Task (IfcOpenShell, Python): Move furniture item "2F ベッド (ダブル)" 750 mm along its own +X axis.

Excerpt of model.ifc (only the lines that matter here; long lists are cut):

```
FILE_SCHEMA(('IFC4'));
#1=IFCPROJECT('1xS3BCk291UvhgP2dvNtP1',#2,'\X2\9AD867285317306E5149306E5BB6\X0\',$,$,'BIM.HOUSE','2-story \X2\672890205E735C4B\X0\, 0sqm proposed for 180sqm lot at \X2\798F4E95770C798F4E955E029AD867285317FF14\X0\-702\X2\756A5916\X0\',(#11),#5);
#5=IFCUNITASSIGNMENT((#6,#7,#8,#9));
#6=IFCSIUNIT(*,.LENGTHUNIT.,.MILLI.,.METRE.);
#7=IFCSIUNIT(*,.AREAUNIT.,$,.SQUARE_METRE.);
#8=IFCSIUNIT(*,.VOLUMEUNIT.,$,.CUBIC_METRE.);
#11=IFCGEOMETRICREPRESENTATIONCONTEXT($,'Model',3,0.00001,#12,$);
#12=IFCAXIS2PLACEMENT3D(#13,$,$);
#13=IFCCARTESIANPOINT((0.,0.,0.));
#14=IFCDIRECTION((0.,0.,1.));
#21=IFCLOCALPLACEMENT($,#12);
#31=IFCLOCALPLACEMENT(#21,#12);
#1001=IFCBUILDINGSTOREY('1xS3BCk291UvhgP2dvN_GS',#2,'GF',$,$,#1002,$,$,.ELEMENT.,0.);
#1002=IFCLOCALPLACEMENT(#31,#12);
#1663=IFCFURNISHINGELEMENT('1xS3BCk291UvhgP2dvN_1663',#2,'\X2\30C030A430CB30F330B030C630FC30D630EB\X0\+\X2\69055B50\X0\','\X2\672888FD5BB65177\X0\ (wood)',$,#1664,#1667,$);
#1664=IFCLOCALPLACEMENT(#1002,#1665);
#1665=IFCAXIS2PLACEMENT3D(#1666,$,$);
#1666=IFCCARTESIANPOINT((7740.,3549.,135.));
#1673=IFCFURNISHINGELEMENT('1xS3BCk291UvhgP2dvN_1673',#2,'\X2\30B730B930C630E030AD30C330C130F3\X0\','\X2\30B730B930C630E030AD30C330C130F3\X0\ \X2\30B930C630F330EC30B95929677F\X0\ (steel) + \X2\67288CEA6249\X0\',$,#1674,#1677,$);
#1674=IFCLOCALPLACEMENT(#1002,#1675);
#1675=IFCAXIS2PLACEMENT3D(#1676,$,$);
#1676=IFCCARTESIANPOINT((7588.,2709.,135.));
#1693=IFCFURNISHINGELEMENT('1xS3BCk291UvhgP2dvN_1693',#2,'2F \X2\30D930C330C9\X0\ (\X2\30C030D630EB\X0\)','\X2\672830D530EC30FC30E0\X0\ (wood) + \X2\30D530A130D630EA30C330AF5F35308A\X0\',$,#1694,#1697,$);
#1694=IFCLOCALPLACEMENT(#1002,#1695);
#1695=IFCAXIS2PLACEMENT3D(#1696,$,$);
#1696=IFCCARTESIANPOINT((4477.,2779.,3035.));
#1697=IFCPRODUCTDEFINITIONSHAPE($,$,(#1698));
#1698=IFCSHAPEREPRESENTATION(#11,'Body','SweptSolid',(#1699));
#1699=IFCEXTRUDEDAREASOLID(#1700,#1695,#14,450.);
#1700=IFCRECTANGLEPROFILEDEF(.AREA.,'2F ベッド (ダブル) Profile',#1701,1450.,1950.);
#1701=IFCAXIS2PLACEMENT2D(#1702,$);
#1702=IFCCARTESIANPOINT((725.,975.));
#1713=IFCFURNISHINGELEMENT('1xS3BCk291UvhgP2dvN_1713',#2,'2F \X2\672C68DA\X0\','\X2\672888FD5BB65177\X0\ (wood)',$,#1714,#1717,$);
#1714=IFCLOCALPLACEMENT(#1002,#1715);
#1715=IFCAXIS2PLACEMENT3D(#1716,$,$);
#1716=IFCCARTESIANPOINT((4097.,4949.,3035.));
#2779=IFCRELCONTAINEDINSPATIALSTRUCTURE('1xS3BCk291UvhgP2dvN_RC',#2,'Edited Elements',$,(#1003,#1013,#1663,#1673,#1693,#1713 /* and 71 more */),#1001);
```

```python
import ifcopenshell
import ifcopenshell.api.geometry
import ifcopenshell.util.placement
import ifcopenshell.util.unit

model = ifcopenshell.open("model.ifc")
unit_scale = ifcopenshell.util.unit.calculate_unit_scale(model)

item = model.by_guid("1xS3BCk291UvhgP2dvN_1693")
matrix = ifcopenshell.util.placement.get_local_placement(item.ObjectPlacement)
matrix[:3, 3] += matrix[:3, 0] * 0.75 / unit_scale
ifcopenshell.api.geometry.edit_object_placement(model, product=item, matrix=matrix, is_si=False)

print(ifcopenshell.util.placement.get_local_placement(item.ObjectPlacement).round(3) + 0.0)

model.write("model_updated.ifc")
```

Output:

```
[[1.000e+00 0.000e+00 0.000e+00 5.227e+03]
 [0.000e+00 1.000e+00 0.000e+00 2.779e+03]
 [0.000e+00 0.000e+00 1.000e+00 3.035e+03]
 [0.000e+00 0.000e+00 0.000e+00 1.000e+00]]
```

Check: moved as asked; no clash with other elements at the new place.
